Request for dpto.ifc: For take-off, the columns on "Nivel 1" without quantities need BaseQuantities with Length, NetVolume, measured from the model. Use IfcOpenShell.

First a look at what the model holds.

```python
import ifcopenshell
import ifcopenshell.util.element
import ifcopenshell.util.unit

model = ifcopenshell.open("dpto.ifc")
print(model.schema)
for unit_type in ("LENGTHUNIT", "AREAUNIT", "VOLUMEUNIT"):
    print(unit_type, ifcopenshell.util.unit.calculate_unit_scale(model, unit_type))
storey = next(s for s in model.by_type("IfcBuildingStorey") if s.Name == "Nivel 1")
columns = [e for e in ifcopenshell.util.element.get_decomposition(storey) if e.is_a("IfcColumn")]
for e in sorted(columns, key=lambda e: e.id()):
    print(e.id(), e.is_a(), e.Name, list(ifcopenshell.util.element.get_psets(e, qtos_only=True)), sep=" | ")
```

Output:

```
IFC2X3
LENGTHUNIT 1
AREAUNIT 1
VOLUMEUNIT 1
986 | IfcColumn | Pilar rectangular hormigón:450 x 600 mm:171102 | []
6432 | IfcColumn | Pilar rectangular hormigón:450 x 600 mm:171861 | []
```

```python
import ifcopenshell
import ifcopenshell.api.pset
import ifcopenshell.geom
import ifcopenshell.util.element
import ifcopenshell.util.shape
import ifcopenshell.util.unit

model = ifcopenshell.open("dpto.ifc")
unit_scale = ifcopenshell.util.unit.calculate_unit_scale(model)
volume_scale = ifcopenshell.util.unit.calculate_unit_scale(model, "VOLUMEUNIT")
settings = ifcopenshell.geom.settings()

storey = next(s for s in model.by_type("IfcBuildingStorey") if s.Name == "Nivel 1")
columns = [e for e in ifcopenshell.util.element.get_decomposition(storey) if e.is_a("IfcColumn")]

for e in sorted(columns, key=lambda e: e.id()):
    if ifcopenshell.util.element.get_psets(e, qtos_only=True, should_inherit=False):
        continue
    # Geometry comes back in metres, in the element's own axes.
    shape = ifcopenshell.geom.create_shape(settings, e)
    values = {
        "Length": ifcopenshell.util.shape.get_z(shape.geometry) / unit_scale,
        "NetVolume": ifcopenshell.util.shape.get_volume(shape.geometry) / volume_scale,
    }
    qto = ifcopenshell.api.pset.add_qto(model, product=e, name="BaseQuantities")
    ifcopenshell.api.pset.edit_qto(model, qto=qto, properties=values)
    print(e.id(), {k: round(v, 3) for k, v in values.items()})

model.write("dpto_edited.ifc")
```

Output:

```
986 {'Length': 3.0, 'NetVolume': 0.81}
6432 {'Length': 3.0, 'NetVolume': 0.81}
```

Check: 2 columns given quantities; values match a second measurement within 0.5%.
